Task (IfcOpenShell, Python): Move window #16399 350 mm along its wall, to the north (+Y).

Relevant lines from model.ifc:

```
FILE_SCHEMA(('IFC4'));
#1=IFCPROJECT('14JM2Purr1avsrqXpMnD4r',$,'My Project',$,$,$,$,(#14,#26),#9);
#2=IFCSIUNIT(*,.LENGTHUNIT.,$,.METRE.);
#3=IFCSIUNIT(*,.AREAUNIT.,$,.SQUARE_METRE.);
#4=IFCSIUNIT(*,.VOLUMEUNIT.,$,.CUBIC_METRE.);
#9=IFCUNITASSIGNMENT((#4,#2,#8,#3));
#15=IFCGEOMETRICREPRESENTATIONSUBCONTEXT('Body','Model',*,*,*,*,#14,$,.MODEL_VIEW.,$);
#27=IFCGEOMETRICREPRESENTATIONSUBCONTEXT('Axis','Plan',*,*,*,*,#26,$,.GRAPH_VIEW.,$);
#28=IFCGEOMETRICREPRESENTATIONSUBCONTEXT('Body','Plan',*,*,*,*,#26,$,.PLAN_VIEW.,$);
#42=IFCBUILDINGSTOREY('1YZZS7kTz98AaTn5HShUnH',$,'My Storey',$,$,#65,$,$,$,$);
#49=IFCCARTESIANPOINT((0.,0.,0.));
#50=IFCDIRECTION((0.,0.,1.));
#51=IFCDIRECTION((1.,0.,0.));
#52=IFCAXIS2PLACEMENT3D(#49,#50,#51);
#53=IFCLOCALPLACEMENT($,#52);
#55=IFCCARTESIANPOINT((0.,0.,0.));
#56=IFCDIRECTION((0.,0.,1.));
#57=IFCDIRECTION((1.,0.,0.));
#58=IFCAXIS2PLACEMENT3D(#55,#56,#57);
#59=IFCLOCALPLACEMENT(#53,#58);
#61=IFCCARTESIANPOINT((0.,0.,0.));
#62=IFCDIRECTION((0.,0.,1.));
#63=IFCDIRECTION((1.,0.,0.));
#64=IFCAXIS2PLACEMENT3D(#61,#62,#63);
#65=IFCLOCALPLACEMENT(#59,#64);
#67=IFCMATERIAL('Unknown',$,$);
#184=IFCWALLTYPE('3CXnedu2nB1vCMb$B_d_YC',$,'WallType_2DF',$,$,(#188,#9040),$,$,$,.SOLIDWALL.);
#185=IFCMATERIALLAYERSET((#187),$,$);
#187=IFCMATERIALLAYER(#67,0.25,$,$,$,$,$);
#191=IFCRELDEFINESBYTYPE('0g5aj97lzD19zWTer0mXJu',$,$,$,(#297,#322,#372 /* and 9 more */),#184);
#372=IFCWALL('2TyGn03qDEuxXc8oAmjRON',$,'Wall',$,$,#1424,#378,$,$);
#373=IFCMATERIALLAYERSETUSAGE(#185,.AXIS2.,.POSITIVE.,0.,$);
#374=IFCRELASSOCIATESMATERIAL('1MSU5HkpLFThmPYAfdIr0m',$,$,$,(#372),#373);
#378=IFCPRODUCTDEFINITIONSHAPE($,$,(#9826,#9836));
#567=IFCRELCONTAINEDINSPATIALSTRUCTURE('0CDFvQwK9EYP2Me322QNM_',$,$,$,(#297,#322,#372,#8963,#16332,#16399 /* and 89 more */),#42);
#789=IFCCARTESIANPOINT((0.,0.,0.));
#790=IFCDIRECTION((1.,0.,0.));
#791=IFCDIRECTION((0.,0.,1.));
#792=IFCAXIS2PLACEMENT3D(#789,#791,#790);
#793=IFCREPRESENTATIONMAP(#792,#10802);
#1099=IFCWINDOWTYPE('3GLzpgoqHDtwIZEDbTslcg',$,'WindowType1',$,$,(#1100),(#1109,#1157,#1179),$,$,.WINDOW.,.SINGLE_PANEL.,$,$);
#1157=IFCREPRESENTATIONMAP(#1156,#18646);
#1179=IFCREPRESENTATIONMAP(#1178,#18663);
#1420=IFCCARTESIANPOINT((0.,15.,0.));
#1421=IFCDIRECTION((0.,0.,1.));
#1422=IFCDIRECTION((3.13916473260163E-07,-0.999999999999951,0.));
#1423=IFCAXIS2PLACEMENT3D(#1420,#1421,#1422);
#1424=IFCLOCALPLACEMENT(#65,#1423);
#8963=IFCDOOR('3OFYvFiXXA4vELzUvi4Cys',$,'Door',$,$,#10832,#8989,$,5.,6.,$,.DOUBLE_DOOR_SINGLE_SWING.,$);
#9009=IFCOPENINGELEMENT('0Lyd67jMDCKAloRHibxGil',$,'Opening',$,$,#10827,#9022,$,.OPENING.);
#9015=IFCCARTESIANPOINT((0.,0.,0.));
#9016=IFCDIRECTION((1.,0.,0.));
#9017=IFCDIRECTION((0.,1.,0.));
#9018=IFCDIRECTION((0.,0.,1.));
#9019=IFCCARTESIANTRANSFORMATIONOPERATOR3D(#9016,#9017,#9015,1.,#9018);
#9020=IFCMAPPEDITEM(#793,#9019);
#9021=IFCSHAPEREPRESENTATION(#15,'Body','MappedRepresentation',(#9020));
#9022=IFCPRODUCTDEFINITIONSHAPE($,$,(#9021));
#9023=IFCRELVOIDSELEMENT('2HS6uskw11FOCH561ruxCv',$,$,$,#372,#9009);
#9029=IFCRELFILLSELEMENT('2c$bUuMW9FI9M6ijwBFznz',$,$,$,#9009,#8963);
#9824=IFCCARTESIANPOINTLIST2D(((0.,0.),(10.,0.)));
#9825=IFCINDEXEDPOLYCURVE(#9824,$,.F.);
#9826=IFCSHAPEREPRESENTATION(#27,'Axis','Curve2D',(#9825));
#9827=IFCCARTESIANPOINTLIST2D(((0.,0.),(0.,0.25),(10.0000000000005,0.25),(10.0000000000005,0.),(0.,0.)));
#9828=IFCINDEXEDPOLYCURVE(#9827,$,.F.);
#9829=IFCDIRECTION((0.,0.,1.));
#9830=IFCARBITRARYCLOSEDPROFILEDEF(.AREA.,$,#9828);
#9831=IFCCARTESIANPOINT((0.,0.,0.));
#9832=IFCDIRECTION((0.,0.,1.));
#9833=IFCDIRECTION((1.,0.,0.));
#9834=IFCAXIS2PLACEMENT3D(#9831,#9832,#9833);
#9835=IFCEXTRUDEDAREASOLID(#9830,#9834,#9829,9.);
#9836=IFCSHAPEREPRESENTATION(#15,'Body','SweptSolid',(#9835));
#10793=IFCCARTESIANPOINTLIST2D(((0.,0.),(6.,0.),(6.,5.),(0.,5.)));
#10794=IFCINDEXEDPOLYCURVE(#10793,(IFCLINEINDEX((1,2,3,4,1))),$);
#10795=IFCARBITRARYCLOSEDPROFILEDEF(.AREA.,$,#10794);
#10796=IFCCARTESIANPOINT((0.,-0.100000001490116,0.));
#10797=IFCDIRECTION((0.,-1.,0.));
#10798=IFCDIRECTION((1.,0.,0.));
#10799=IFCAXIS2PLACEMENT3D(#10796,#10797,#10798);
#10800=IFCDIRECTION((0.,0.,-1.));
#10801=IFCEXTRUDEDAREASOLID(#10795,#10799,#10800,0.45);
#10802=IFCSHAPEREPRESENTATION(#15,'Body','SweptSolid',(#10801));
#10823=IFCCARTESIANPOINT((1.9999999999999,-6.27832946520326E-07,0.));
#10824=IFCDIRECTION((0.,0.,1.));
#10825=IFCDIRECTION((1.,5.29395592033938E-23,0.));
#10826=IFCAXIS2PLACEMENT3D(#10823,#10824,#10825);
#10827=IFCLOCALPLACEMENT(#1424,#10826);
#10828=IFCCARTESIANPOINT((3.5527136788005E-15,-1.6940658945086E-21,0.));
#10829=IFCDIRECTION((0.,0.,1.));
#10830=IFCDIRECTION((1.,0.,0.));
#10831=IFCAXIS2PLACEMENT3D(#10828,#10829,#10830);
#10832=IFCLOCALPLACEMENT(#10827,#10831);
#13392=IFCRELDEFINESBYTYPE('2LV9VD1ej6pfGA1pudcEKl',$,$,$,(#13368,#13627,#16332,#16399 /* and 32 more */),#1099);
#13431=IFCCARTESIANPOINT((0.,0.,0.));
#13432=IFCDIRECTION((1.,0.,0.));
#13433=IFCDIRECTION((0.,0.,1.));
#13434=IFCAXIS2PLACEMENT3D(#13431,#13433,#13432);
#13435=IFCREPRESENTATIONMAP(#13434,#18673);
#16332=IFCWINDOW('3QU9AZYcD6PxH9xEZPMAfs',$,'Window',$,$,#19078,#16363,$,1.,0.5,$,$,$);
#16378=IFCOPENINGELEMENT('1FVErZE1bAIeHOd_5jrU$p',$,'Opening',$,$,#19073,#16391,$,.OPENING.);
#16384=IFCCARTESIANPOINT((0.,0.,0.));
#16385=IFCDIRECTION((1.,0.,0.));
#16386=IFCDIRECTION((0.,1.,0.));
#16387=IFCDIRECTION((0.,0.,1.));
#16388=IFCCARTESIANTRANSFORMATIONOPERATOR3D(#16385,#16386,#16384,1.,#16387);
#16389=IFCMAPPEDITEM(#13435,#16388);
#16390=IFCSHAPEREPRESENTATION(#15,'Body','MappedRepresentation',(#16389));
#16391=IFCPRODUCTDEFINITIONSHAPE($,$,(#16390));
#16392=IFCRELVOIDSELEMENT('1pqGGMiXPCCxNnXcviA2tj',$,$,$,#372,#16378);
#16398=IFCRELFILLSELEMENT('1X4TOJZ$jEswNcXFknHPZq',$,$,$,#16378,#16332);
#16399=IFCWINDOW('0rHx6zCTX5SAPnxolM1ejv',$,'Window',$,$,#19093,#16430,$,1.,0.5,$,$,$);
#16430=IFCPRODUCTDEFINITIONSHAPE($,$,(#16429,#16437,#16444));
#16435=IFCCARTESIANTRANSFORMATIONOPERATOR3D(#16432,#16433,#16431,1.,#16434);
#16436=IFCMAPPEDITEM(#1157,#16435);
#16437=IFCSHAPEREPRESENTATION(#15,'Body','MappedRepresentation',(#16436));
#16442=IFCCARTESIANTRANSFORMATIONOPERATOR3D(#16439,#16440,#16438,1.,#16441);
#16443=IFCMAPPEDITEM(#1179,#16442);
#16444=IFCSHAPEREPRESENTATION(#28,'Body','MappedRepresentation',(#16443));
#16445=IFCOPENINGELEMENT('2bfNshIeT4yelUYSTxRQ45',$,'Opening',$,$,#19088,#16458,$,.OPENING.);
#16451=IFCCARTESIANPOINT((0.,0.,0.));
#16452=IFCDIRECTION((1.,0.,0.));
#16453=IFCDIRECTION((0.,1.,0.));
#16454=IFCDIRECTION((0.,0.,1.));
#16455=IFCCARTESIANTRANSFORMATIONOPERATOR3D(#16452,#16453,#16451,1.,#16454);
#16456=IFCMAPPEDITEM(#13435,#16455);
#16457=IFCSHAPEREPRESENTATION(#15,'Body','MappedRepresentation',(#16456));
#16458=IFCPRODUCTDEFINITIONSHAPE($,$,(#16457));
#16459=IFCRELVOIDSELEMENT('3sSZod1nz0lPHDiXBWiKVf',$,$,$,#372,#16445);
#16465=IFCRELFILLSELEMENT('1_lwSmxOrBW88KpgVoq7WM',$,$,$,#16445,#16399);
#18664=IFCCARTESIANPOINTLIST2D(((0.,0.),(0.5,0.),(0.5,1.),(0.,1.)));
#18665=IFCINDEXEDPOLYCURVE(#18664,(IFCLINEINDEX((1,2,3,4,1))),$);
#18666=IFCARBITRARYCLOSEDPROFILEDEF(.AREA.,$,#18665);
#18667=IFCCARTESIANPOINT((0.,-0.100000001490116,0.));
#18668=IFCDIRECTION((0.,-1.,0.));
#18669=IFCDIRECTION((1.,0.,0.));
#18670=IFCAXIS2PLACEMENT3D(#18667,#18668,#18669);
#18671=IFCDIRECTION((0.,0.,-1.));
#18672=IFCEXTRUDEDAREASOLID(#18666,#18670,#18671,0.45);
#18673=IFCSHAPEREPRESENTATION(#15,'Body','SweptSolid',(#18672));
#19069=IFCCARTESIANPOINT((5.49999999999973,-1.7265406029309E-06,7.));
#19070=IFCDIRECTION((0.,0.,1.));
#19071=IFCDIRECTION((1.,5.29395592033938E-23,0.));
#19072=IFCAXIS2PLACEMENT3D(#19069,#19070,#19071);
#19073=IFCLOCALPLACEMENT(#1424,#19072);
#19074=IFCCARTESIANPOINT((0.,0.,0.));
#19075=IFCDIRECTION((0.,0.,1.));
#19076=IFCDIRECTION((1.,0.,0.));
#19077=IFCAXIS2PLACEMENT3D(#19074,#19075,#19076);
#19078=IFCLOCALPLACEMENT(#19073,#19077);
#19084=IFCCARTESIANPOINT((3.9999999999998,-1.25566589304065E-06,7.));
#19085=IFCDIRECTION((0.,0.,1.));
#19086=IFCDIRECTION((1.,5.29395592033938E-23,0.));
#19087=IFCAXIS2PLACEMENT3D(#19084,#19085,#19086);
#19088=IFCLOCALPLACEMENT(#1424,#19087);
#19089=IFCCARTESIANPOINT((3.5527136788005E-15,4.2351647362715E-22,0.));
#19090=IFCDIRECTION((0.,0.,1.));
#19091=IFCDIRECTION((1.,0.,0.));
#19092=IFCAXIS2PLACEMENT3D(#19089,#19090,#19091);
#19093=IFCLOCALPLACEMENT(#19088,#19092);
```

```python
import ifcopenshell
import ifcopenshell.api.geometry
import ifcopenshell.util.placement
import ifcopenshell.util.unit

model = ifcopenshell.open("model.ifc")
unit_scale = ifcopenshell.util.unit.calculate_unit_scale(model)

window = model.by_guid("0rHx6zCTX5SAPnxolM1ejv")
opening = window.FillsVoids[0].RelatingOpeningElement
wall = opening.VoidsElements[0].RelatingBuildingElement

wall_matrix = ifcopenshell.util.placement.get_local_placement(wall.ObjectPlacement)
shift = wall_matrix[:3, 0] * -0.35 / unit_scale
before = ifcopenshell.util.placement.get_local_placement(window.ObjectPlacement)[:3, 3].copy()

# The window is placed relative to its opening, so it follows when the opening moves.
matrix = ifcopenshell.util.placement.get_local_placement(opening.ObjectPlacement)
matrix[:3, 3] += shift
ifcopenshell.api.geometry.edit_object_placement(
    model, product=opening, matrix=matrix, is_si=False, should_transform_children=True
)

after = ifcopenshell.util.placement.get_local_placement(window.ObjectPlacement)[:3, 3]
print("window moved by", (after - before).round(3) + 0.0)

model.write("model_updated.ifc")
```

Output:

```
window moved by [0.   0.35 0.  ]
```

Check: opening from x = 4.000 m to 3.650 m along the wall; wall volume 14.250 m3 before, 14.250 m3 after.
